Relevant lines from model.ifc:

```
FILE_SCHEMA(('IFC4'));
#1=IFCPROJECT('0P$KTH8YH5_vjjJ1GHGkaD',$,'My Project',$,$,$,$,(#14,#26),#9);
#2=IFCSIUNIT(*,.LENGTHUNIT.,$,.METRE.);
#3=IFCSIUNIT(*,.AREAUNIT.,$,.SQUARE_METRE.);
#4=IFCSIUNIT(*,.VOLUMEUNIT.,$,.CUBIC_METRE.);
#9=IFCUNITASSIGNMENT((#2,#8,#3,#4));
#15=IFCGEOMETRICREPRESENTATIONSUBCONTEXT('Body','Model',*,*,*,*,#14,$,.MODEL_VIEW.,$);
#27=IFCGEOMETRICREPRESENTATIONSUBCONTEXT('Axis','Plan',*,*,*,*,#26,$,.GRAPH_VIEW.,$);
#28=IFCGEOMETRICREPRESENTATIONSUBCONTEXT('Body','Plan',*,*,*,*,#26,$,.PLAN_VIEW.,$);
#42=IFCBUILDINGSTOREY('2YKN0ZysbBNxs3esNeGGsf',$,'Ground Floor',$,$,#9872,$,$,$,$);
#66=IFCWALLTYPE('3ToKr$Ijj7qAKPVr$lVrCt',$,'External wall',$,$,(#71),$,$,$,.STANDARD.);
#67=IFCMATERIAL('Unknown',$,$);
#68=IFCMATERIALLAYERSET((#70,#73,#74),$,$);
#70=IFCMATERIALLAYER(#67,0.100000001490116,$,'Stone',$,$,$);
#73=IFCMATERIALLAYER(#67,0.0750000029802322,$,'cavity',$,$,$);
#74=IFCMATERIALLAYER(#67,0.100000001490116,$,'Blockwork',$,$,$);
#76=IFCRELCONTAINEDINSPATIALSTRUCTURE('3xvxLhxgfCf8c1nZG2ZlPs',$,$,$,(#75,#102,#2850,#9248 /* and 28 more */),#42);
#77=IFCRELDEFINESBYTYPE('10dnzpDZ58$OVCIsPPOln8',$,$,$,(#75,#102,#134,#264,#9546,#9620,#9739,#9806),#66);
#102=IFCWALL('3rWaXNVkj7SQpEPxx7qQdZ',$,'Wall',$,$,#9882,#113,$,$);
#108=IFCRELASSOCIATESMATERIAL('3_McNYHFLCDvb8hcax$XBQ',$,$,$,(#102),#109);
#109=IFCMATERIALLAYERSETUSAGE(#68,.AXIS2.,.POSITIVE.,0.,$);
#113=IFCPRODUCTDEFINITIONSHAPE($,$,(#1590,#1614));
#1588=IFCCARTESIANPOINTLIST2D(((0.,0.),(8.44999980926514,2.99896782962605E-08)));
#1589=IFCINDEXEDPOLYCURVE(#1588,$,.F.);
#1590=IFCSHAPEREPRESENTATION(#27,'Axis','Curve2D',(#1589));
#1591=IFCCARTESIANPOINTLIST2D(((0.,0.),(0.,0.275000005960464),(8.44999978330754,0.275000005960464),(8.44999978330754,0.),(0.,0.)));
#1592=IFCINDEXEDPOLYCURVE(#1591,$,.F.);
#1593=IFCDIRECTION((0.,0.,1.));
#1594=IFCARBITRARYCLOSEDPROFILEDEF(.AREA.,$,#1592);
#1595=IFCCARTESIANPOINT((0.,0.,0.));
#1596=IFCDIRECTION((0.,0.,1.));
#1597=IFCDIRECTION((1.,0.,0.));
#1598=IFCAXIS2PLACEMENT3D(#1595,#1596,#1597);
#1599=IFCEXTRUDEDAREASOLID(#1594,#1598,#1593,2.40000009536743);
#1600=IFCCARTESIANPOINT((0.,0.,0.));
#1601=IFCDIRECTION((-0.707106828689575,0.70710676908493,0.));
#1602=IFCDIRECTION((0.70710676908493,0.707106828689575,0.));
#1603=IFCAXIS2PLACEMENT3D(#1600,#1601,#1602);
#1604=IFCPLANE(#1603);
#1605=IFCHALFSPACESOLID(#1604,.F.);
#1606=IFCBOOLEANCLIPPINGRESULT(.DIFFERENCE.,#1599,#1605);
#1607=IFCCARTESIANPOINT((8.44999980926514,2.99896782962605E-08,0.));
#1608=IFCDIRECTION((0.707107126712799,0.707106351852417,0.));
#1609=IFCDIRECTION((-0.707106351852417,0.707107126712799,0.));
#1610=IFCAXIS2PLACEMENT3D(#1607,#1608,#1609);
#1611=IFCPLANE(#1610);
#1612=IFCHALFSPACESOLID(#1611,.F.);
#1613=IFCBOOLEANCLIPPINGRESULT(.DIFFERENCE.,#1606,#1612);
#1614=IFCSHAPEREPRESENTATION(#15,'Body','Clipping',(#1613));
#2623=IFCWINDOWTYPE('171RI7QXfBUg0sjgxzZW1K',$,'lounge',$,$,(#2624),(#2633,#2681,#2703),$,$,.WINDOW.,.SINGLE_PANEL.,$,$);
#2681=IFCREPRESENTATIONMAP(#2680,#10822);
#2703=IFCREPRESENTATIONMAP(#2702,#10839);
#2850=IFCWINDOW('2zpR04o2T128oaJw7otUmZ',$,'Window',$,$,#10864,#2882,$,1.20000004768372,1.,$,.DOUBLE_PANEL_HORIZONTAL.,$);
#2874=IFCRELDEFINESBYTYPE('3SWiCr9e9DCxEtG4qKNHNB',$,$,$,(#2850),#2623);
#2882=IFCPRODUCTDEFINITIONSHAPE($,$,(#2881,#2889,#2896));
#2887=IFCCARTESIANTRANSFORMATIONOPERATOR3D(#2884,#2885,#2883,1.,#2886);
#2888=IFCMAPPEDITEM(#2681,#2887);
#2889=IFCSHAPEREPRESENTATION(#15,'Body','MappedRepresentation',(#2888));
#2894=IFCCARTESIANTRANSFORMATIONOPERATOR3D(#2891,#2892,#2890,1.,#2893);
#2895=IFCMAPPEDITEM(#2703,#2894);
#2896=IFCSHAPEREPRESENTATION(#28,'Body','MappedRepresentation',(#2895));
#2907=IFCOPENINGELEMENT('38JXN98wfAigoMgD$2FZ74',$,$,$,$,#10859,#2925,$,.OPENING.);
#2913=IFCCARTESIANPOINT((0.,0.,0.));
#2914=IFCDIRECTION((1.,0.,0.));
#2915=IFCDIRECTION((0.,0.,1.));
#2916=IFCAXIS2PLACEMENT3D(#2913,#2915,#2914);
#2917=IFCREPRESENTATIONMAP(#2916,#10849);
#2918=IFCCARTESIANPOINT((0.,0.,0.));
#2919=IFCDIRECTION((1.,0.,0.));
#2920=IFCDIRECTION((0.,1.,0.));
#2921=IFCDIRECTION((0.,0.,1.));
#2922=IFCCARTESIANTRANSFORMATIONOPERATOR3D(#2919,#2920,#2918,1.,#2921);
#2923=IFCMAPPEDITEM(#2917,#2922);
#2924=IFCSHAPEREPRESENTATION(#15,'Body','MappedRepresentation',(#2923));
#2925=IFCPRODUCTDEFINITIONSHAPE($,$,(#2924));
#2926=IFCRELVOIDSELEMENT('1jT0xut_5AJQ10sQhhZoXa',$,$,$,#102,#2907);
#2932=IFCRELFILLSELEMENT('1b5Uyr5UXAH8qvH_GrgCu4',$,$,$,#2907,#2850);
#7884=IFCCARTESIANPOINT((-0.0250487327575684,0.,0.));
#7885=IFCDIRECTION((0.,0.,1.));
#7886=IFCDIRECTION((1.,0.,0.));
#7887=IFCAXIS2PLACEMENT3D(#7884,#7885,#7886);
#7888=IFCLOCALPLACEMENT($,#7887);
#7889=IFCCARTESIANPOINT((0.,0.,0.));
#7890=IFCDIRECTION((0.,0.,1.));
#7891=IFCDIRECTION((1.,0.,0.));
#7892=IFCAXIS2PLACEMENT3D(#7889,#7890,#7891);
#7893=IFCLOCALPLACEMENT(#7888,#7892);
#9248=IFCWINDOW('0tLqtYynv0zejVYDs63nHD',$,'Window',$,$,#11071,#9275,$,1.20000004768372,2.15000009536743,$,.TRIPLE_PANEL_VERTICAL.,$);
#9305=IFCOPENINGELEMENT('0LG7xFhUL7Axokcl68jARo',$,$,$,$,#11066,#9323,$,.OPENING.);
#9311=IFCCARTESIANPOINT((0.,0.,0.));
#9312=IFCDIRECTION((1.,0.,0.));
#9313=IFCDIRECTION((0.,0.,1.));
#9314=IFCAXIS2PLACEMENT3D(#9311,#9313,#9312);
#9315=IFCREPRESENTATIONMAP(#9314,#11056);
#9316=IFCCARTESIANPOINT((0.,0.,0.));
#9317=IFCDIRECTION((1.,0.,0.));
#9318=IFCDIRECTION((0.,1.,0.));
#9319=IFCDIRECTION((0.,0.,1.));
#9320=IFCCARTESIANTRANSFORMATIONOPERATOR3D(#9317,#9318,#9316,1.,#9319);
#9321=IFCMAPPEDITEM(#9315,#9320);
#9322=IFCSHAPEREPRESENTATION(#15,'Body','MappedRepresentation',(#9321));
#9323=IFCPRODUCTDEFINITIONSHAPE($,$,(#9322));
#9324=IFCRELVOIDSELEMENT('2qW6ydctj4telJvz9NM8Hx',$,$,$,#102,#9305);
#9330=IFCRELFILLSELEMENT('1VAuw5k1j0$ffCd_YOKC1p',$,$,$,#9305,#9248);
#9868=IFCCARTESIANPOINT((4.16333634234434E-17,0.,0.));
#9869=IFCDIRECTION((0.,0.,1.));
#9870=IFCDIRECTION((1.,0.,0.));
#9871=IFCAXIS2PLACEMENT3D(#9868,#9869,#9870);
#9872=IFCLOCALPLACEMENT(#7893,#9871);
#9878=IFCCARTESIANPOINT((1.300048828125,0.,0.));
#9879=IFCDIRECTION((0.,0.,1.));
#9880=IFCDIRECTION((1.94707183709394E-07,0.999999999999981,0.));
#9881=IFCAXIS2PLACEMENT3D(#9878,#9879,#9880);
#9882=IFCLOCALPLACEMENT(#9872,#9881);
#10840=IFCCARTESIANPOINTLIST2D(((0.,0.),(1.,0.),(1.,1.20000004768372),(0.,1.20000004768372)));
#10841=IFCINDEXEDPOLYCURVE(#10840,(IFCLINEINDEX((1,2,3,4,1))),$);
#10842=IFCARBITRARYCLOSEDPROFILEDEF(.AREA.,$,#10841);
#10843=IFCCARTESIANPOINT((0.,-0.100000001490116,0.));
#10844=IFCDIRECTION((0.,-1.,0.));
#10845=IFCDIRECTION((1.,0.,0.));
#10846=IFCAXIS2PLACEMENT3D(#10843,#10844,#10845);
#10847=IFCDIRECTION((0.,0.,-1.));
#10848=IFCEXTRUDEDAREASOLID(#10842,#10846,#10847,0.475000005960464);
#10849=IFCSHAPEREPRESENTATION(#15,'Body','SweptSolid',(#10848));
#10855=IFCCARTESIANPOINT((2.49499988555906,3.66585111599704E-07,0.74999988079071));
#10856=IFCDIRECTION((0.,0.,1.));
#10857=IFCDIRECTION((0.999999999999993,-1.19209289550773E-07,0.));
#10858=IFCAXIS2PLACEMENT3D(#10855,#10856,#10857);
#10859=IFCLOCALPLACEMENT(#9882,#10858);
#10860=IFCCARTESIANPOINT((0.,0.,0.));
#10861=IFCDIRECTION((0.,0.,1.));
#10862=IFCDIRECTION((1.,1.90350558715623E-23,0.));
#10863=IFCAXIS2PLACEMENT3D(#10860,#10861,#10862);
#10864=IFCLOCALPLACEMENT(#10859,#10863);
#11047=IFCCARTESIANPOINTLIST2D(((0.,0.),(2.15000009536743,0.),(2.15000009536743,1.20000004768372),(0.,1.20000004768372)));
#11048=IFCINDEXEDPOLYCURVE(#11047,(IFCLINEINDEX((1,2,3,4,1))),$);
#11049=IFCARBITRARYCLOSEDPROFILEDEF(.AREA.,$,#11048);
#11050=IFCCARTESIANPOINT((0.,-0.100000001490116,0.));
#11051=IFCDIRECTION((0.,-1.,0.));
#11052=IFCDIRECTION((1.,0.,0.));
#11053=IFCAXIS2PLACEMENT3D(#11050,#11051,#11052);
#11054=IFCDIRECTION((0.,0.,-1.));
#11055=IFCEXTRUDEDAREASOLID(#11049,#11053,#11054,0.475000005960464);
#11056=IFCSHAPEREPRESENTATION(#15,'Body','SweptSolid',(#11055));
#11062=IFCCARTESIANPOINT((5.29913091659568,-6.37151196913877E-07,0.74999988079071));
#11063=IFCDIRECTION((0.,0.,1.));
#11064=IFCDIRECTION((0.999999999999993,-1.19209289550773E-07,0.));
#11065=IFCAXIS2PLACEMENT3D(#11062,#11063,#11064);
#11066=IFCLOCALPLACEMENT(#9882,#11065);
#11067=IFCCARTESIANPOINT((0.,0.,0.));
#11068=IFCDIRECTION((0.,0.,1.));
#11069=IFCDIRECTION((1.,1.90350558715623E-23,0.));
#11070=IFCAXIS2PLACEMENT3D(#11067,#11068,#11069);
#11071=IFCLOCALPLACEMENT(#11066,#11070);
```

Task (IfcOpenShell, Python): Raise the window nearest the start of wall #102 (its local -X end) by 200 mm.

```python
import numpy as np
import ifcopenshell
import ifcopenshell.api.geometry
import ifcopenshell.util.placement
import ifcopenshell.util.unit

model = ifcopenshell.open("model.ifc")
unit_scale = ifcopenshell.util.unit.calculate_unit_scale(model)

window = model.by_guid("2zpR04o2T128oaJw7otUmZ")
opening = window.FillsVoids[0].RelatingOpeningElement
dz = 0.2 / unit_scale

shift = np.array([0.0, 0.0, dz])
# The window is placed relative to its opening, so it follows when the opening moves.
matrix = ifcopenshell.util.placement.get_local_placement(opening.ObjectPlacement)
matrix[:3, 3] += shift
ifcopenshell.api.geometry.edit_object_placement(
    model, product=opening, matrix=matrix, is_si=False, should_transform_children=True
)

print(f"moved by {dz * unit_scale:+.3f} m")

model.write("model_rev.ifc")
```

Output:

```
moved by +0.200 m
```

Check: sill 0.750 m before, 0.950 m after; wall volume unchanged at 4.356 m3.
